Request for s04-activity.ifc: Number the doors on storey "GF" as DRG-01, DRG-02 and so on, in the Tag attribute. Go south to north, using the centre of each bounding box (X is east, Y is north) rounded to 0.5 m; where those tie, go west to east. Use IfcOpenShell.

First a look at what the model holds.

```python
import ifcopenshell
import ifcopenshell.util.element
import ifcopenshell.util.placement

model = ifcopenshell.open("s04-activity.ifc")
print(model.schema)
storey = next(s for s in model.by_type("IfcBuildingStorey") if s.Name == "GF")
doors = [e for e in ifcopenshell.util.element.get_decomposition(storey) if e.is_a("IfcDoor")]
for e in sorted(doors, key=lambda e: e.id()):
    origin = ifcopenshell.util.placement.get_local_placement(e.ObjectPlacement)[:3, 3]
    print(e.id(), e.Tag, e.Name, origin.round(2) + 0.0, sep=" | ")
```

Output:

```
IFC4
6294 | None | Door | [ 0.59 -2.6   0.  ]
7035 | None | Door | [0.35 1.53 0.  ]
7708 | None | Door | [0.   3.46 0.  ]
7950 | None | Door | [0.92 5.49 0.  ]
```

```python
import ifcopenshell
import ifcopenshell.geom
import ifcopenshell.util.element
import ifcopenshell.util.shape

model = ifcopenshell.open("s04-activity.ifc")
settings = ifcopenshell.geom.settings()
settings.set("use-world-coords", True)


def centre(element):
    shape = ifcopenshell.geom.create_shape(settings, element)
    return ifcopenshell.util.shape.get_bbox_centroid(shape.geometry)


storey = next(s for s in model.by_type("IfcBuildingStorey") if s.Name == "GF")
doors = [e for e in ifcopenshell.util.element.get_decomposition(storey) if e.is_a("IfcDoor")]

# Insertion points can sit at a corner or the storey origin, so sort by the geometry (in metres).
centres = {e: centre(e) for e in doors}
doors.sort(key=lambda e: (round(centres[e][1] / 0.5), centres[e][0]))

for i, e in enumerate(doors, start=1):
    number = f"DRG-{i:02d}"
    e.Tag = number
    print(e.id(), number)

model.write("s04-activity_rev.ifc")
```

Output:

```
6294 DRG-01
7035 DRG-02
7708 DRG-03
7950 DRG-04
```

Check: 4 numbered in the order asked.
